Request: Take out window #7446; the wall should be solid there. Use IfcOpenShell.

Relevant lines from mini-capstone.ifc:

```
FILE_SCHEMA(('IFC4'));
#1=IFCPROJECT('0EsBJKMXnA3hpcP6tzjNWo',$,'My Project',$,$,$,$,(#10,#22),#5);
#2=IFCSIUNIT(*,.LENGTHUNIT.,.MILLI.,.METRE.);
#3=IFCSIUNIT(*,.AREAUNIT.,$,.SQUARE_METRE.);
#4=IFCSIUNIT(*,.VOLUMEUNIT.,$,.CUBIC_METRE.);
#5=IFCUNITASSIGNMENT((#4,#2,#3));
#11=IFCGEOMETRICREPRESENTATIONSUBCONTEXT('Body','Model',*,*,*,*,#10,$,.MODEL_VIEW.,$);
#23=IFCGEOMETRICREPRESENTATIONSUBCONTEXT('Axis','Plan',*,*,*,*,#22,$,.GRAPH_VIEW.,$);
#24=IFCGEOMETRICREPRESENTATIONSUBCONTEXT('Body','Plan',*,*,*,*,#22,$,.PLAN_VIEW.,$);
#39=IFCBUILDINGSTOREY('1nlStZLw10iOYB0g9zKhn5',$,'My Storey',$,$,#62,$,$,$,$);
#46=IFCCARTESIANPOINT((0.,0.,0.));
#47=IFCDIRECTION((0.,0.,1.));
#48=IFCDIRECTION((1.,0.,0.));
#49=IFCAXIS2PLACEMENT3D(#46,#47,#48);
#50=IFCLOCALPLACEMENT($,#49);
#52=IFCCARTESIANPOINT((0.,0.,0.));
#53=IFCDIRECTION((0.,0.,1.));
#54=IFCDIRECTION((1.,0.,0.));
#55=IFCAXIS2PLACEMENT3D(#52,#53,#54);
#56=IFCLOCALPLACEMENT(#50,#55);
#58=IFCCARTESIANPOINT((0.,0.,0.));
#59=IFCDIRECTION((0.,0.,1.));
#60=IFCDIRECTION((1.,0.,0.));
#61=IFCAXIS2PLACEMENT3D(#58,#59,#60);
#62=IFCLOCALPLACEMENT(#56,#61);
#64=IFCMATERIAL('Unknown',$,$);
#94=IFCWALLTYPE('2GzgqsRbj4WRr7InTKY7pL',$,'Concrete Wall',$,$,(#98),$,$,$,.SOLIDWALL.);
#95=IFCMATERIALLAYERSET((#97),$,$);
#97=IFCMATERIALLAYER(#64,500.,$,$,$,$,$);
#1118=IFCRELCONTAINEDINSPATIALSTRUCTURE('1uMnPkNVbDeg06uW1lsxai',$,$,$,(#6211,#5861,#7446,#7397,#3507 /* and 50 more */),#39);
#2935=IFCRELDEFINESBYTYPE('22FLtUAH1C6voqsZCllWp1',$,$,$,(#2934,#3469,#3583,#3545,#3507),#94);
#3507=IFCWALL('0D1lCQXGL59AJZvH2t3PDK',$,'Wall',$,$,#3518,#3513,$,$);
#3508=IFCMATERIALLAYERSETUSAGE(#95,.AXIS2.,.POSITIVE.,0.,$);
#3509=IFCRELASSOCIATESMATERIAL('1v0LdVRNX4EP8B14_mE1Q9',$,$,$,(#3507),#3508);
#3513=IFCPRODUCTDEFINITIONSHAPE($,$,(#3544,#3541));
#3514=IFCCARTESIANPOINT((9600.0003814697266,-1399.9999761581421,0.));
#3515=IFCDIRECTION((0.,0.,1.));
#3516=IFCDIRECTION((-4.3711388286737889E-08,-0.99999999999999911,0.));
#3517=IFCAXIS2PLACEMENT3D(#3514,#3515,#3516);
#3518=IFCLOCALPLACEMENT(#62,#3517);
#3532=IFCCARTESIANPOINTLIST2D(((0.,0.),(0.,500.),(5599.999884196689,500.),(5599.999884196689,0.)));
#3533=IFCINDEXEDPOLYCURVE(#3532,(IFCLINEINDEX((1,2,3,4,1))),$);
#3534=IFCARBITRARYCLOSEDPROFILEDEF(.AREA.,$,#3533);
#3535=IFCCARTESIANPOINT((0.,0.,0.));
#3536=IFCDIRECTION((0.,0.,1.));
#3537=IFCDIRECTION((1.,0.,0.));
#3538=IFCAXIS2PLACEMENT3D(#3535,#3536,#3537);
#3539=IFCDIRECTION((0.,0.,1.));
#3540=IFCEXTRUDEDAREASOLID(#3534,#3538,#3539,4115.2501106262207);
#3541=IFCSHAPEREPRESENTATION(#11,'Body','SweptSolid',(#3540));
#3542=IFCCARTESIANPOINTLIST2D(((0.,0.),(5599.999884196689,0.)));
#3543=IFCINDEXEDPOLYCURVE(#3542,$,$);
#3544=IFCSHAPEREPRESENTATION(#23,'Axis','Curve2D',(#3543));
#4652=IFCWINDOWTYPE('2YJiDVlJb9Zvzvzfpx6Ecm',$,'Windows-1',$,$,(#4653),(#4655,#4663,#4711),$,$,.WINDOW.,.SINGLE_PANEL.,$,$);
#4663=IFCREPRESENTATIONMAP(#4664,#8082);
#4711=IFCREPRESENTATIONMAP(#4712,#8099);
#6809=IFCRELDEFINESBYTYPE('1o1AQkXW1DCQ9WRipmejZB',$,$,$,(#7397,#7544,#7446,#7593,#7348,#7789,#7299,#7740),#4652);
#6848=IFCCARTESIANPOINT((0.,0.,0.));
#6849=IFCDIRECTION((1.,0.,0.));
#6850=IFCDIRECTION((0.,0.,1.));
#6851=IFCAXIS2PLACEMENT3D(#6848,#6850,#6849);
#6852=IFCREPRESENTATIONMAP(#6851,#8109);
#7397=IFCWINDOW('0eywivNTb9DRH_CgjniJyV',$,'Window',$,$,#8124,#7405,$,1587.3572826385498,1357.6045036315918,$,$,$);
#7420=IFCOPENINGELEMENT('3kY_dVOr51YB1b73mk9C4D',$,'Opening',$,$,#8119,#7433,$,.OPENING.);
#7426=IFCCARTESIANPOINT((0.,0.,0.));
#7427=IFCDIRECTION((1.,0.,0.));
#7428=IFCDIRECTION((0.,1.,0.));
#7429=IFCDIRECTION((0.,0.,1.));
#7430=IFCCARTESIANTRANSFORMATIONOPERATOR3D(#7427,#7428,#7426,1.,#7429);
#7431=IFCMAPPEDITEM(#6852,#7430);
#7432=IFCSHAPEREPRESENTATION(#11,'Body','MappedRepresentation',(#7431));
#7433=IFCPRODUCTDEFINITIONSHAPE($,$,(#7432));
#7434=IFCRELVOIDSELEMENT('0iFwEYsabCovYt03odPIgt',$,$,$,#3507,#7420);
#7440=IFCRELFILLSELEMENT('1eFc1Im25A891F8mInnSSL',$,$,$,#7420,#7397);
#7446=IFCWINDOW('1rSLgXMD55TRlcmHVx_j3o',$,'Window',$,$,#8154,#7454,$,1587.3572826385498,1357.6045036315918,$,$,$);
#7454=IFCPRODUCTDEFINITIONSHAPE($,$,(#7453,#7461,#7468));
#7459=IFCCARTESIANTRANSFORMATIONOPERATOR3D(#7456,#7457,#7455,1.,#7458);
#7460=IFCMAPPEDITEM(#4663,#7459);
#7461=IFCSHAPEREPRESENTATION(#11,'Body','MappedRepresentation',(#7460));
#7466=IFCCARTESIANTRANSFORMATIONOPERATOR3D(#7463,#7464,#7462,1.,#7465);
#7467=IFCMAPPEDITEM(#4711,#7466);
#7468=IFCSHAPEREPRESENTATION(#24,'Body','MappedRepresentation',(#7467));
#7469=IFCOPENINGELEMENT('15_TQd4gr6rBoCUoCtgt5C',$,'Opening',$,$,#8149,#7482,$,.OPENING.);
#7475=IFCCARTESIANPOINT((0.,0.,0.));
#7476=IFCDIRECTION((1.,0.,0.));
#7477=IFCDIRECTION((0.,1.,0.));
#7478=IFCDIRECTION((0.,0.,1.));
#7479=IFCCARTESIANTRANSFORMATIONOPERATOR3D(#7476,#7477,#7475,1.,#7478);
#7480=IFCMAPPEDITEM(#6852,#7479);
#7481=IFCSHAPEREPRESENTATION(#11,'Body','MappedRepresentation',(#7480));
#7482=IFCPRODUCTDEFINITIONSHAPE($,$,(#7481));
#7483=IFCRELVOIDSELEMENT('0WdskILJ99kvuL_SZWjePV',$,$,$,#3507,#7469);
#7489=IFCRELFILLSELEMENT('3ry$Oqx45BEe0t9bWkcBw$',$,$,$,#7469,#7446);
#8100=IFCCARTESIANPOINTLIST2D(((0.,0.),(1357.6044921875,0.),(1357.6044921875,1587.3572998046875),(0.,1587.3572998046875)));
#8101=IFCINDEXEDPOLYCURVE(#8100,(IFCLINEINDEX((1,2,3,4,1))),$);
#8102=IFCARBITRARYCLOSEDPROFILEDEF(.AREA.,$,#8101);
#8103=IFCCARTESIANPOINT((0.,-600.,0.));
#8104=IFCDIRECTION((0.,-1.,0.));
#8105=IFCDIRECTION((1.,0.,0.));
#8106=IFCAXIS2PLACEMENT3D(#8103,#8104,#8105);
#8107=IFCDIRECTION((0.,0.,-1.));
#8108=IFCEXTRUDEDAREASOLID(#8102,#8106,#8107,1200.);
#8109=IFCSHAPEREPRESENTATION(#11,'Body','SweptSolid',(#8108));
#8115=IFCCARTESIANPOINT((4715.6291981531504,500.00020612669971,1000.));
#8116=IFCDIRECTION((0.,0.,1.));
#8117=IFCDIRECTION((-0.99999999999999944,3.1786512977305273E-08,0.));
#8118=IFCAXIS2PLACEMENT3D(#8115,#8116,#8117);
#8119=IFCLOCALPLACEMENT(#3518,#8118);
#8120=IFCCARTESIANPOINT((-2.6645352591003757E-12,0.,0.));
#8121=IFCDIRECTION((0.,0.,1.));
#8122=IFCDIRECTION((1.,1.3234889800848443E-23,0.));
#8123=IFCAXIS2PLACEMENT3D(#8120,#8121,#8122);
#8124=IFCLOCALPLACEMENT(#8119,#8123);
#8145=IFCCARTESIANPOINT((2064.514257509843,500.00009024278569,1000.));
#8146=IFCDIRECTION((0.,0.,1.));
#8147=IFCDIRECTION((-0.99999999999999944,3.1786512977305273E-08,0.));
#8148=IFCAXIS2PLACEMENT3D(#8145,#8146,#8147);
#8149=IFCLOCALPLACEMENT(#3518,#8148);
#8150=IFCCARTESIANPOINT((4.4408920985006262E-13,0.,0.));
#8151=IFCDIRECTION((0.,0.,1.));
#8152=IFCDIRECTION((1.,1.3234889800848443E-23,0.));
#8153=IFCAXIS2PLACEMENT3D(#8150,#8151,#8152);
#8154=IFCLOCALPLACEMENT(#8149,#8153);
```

```python
import ifcopenshell
import ifcopenshell.api.feature
import ifcopenshell.api.root
import ifcopenshell.geom
import ifcopenshell.util.shape

model = ifcopenshell.open("mini-capstone.ifc")
settings = ifcopenshell.geom.settings()


def volume(element):
    """Net volume in cubic metres, openings subtracted."""
    shape = ifcopenshell.geom.create_shape(settings, element)
    return ifcopenshell.util.shape.get_volume(shape.geometry)


window = model.by_id(7446)
opening = window.FillsVoids[0].RelatingOpeningElement
wall = opening.VoidsElements[0].RelatingBuildingElement
before = volume(wall)

ifcopenshell.api.root.remove_product(model, product=window)
ifcopenshell.api.feature.remove_feature(model, feature=opening)

after = volume(wall)

print(f"wall volume {before:.3f} -> {after:.3f} m3")

model.write("mini-capstone_rev.ifc")
```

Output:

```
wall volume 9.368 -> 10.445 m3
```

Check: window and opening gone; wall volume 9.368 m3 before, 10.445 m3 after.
